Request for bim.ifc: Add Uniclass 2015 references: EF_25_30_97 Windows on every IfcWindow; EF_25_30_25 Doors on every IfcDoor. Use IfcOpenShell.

First a look at what the model holds.

```python
import ifcopenshell

model = ifcopenshell.open("bim.ifc")
print(model.schema)
print("classifications:", [c.Name for c in model.by_type("IfcClassification")])
for ifc_class in ("IfcDoor", "IfcRoof", "IfcStair", "IfcWall", "IfcWindow"):
    print(ifc_class, len(model.by_type(ifc_class)))
```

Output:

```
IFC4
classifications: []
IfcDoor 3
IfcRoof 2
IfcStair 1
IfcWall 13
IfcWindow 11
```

```python
import ifcopenshell
import ifcopenshell.api.classification

model = ifcopenshell.open("bim.ifc")

system = ifcopenshell.api.classification.add_classification(model, classification="Uniclass 2015")

codes = {
    "IfcWindow": ("EF_25_30_97", "Windows"),
    "IfcDoor": ("EF_25_30_25", "Doors"),
}
for ifc_class, (code, name) in codes.items():
    products = model.by_type(ifc_class)
    ifcopenshell.api.classification.add_reference(
        model, products=products, classification=system, identification=code, name=name
    )
    print(code, len(products))

model.write("bim_updated.ifc")
```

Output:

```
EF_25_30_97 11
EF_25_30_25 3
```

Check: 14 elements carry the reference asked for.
